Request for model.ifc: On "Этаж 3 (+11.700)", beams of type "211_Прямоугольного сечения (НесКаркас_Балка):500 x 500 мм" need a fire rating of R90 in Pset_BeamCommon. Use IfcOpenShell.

First a look at what the model holds.

```python
import ifcopenshell
import ifcopenshell.util.element

model = ifcopenshell.open("model.ifc")
print(model.schema)
storey = next(s for s in model.by_type("IfcBuildingStorey") if s.Name == "Этаж 3 (+11.700)")
beams = [e for e in ifcopenshell.util.element.get_decomposition(storey) if e.is_a("IfcBeam")]
seen = {}
for e in beams:
    element_type = ifcopenshell.util.element.get_type(e)
    key = (element_type.Name if element_type != e and element_type else None, ifcopenshell.util.element.get_pset(e, "Pset_BeamCommon", "FireRating"))
    seen[key] = seen.get(key, 0) + 1
for (name, value), count in sorted(seen.items(), key=str):
    print(count, "x", name, "|", value)
```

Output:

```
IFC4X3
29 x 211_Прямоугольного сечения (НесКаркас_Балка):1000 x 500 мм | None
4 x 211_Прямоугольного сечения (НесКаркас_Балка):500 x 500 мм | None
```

```python
import ifcopenshell
import ifcopenshell.api.pset
import ifcopenshell.util.element

model = ifcopenshell.open("model.ifc")

storey = next(s for s in model.by_type("IfcBuildingStorey") if s.Name == "Этаж 3 (+11.700)")
beams = [e for e in ifcopenshell.util.element.get_decomposition(storey) if e.is_a("IfcBeam")]

count = 0
for e in beams:
    element_type = ifcopenshell.util.element.get_type(e)
    if element_type in (None, e) or element_type.Name != "211_Прямоугольного сечения (НесКаркас_Балка):500 x 500 мм":
        continue
    # add_pset returns the element's existing set when there is one.
    pset = ifcopenshell.api.pset.add_pset(model, product=e, name="Pset_BeamCommon")
    ifcopenshell.api.pset.edit_pset(model, pset=pset, properties={"FireRating": "R90"})
    count += 1

print(count, "beams updated")

model.write("model_v2.ifc")
```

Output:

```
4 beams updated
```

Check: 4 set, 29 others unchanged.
